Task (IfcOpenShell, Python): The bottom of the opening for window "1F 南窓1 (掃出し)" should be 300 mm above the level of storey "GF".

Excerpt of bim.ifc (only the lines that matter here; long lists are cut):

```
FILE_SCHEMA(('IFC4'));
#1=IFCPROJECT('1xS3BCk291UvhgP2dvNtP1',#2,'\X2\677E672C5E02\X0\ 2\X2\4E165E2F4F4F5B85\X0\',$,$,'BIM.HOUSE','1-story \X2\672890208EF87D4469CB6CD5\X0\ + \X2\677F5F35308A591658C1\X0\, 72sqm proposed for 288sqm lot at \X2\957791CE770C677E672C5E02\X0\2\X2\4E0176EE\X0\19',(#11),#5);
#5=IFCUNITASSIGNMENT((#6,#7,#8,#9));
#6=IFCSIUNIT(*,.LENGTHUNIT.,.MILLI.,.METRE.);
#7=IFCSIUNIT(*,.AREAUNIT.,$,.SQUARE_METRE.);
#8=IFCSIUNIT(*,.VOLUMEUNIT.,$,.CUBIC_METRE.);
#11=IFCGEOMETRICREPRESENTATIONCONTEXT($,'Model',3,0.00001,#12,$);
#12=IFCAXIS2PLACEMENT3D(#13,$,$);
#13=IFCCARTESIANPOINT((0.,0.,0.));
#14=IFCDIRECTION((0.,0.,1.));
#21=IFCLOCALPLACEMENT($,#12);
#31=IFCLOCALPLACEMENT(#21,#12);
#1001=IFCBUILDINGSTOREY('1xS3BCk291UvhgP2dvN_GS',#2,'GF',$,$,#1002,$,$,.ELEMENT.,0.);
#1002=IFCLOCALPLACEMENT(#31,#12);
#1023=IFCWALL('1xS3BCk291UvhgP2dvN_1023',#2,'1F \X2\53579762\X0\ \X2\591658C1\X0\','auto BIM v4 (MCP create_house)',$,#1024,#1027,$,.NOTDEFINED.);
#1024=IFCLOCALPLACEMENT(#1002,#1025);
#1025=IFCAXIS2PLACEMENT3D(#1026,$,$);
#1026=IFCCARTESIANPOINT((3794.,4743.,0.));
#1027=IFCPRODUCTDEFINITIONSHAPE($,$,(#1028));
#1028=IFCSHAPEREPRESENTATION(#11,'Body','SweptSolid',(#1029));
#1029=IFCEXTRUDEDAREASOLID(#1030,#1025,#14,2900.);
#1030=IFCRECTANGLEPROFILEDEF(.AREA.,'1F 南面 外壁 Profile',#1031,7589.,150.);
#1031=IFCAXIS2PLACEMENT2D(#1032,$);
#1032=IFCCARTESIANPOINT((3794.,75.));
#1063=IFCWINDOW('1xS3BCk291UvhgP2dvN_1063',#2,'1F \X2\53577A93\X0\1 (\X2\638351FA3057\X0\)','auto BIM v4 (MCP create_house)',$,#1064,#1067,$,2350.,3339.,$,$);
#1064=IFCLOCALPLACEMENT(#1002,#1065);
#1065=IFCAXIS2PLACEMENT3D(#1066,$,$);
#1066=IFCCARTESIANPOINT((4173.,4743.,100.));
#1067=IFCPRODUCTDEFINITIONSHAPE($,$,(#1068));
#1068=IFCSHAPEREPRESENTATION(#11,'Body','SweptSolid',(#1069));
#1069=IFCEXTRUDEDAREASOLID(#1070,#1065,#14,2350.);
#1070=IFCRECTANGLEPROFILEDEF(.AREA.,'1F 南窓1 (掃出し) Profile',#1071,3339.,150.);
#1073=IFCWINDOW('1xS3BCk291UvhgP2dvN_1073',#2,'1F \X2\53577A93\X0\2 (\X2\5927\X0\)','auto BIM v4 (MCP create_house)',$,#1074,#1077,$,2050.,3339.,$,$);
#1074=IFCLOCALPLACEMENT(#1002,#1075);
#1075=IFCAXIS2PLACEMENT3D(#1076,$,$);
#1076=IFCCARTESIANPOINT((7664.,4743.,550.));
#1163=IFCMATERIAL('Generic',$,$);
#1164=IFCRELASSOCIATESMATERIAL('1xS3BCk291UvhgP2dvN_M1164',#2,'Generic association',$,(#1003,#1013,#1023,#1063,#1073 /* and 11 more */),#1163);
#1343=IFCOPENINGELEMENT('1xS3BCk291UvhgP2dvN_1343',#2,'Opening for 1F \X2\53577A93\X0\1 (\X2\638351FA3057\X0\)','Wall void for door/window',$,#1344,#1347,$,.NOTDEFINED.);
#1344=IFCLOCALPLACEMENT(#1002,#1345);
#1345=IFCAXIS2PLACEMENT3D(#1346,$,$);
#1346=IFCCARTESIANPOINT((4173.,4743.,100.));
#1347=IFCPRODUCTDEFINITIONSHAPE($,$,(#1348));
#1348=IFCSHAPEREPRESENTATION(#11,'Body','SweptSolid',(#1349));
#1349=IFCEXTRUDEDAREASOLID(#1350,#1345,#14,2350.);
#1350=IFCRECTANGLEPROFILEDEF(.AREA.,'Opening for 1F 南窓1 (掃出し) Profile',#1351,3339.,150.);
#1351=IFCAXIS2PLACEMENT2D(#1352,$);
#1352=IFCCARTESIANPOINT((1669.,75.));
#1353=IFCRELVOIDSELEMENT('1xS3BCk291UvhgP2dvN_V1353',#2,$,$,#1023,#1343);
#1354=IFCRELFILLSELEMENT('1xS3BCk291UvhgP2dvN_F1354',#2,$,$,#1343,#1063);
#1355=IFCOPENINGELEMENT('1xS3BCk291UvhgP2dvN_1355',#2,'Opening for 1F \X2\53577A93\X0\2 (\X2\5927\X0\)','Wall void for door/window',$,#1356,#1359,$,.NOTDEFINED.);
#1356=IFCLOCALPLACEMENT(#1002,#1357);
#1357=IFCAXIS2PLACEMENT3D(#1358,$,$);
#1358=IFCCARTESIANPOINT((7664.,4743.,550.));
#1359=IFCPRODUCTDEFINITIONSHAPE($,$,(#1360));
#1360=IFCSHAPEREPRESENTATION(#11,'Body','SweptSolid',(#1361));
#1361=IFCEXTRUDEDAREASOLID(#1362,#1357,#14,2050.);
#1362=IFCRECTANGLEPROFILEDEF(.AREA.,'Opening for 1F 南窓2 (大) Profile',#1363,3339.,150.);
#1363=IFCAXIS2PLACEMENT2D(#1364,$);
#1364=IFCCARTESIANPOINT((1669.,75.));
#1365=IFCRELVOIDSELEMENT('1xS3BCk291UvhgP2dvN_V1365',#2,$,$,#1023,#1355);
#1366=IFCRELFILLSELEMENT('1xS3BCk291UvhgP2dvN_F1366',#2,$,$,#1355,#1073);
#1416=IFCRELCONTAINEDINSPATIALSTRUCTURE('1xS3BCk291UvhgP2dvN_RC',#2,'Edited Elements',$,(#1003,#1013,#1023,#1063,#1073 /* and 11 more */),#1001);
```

```python
import numpy as np
import ifcopenshell
import ifcopenshell.api.geometry
import ifcopenshell.geom
import ifcopenshell.util.element
import ifcopenshell.util.placement
import ifcopenshell.util.shape
import ifcopenshell.util.unit

model = ifcopenshell.open("bim.ifc")
unit_scale = ifcopenshell.util.unit.calculate_unit_scale(model)

window = model.by_guid("1xS3BCk291UvhgP2dvN_1063")
opening = window.FillsVoids[0].RelatingOpeningElement
storey = ifcopenshell.util.element.get_container(window, ifc_class="IfcBuildingStorey")
level = ifcopenshell.util.placement.get_local_placement(storey.ObjectPlacement)[2, 3]

# The opening's origin need not be at the sill, so measure its lowest point.
shape = ifcopenshell.geom.create_shape(ifcopenshell.geom.settings(), opening)
bottom = ifcopenshell.util.shape.get_shape_bottom_elevation(shape, shape.geometry) / unit_scale
dz = level + 0.3 / unit_scale - bottom

shift = np.array([0.0, 0.0, dz])
# The window is not placed relative to its opening, so move both.
for product in (opening, window):
    matrix = ifcopenshell.util.placement.get_local_placement(product.ObjectPlacement)
    matrix[:3, 3] += shift
    ifcopenshell.api.geometry.edit_object_placement(model, product=product, matrix=matrix, is_si=False)

print(f"moved by {dz * unit_scale:+.3f} m")

model.write("bim_rev.ifc")
```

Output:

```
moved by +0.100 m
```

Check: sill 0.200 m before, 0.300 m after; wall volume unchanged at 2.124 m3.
